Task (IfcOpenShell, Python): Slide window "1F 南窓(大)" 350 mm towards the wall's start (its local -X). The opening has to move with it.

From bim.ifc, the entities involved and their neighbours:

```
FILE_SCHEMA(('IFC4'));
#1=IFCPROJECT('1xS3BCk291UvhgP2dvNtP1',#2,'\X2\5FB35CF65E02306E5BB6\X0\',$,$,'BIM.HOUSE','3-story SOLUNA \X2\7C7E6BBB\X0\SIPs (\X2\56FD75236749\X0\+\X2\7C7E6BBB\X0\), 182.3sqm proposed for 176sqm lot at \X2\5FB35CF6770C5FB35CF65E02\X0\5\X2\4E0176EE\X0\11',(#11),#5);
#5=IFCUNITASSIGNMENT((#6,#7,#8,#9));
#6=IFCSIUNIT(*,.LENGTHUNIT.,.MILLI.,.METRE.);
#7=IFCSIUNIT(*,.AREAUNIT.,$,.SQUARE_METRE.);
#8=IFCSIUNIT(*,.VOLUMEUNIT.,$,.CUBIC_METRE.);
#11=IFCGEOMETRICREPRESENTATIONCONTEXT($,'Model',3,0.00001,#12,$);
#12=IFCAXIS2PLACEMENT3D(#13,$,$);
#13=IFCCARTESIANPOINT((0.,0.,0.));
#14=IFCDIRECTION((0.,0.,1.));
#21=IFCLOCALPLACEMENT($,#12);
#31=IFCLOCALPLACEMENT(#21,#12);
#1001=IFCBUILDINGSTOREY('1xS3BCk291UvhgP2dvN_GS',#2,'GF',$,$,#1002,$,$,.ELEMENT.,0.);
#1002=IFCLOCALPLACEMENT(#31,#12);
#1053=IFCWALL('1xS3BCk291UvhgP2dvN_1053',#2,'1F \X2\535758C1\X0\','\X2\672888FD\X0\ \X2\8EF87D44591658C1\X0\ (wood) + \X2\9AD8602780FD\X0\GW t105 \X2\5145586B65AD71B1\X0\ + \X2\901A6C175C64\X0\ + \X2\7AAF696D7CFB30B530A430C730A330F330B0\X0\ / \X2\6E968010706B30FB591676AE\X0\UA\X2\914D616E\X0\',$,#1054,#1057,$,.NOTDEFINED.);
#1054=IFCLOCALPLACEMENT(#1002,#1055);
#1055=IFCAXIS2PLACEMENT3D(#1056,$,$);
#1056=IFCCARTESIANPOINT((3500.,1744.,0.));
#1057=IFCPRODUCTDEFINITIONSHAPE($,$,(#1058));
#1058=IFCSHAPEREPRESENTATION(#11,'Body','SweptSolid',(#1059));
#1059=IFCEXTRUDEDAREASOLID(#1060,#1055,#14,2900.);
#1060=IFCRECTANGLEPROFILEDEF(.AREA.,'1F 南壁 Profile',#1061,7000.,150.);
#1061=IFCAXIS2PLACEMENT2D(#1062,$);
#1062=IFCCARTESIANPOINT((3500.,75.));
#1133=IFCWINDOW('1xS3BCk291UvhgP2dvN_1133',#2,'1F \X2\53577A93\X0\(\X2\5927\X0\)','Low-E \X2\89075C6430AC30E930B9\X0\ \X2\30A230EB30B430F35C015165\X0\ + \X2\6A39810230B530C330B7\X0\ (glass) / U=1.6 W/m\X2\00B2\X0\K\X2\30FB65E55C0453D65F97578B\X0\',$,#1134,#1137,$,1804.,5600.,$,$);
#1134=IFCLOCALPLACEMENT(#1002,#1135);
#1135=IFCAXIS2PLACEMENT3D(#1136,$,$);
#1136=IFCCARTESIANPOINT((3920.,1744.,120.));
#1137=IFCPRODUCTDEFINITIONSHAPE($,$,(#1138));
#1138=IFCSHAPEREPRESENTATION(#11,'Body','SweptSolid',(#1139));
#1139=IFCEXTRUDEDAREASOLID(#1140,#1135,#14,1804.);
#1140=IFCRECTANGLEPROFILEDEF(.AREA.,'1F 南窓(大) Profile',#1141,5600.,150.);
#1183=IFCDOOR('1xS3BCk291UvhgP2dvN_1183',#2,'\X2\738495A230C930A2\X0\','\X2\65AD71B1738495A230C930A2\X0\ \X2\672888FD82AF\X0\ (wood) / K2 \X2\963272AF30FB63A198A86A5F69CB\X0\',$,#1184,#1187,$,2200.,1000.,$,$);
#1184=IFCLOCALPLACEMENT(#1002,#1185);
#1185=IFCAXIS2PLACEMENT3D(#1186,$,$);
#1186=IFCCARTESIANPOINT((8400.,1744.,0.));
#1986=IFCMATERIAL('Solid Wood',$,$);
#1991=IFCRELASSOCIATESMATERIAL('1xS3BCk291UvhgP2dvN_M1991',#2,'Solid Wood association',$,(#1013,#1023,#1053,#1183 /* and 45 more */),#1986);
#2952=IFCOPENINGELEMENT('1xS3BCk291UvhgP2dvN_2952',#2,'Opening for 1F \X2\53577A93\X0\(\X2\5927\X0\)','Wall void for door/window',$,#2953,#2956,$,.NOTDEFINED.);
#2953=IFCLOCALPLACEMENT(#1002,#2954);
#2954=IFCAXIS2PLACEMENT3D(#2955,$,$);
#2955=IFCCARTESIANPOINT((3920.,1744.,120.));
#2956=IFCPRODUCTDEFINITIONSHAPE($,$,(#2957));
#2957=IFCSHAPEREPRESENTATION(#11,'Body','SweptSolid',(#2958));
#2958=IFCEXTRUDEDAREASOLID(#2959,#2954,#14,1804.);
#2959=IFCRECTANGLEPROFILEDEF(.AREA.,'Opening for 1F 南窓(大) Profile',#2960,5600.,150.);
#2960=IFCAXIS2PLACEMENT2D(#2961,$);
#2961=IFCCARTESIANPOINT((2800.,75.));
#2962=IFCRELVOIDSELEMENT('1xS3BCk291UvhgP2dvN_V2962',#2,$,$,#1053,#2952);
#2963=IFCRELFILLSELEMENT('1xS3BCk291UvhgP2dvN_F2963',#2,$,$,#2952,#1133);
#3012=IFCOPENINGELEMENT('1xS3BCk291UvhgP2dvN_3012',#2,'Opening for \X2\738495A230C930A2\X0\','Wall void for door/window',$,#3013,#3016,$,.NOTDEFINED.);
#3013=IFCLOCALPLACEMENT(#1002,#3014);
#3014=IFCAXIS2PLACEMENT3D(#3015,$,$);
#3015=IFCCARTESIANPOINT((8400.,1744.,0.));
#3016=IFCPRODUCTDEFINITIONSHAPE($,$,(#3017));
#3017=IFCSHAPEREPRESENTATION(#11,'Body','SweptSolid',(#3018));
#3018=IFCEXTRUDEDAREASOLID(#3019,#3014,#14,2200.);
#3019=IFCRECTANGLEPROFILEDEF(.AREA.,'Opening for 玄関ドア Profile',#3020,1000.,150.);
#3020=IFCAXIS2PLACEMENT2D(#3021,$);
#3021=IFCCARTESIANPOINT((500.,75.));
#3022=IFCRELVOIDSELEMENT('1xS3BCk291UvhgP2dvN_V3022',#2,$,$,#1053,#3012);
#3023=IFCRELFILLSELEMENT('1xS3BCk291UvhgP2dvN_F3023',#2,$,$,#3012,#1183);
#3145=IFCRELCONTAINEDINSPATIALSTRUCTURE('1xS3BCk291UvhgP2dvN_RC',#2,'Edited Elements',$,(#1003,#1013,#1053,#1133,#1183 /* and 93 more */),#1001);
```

```python
import ifcopenshell
import ifcopenshell.api.geometry
import ifcopenshell.util.placement

model = ifcopenshell.open("bim.ifc")

window = model.by_guid("1xS3BCk291UvhgP2dvN_1133")
opening = window.FillsVoids[0].RelatingOpeningElement
wall = opening.VoidsElements[0].RelatingBuildingElement

wall_matrix = ifcopenshell.util.placement.get_local_placement(wall.ObjectPlacement)
shift = wall_matrix[:3, 0] * -350.0
before = ifcopenshell.util.placement.get_local_placement(window.ObjectPlacement)[:3, 3].copy()

# The window is not placed relative to its opening, so move both.
for product in (opening, window):
    matrix = ifcopenshell.util.placement.get_local_placement(product.ObjectPlacement)
    matrix[:3, 3] += shift
    ifcopenshell.api.geometry.edit_object_placement(model, product=product, matrix=matrix, is_si=False)

after = ifcopenshell.util.placement.get_local_placement(window.ObjectPlacement)[:3, 3]
print("window moved by", (after - before).round(3) + 0.0)

model.write("bim_rev.ifc")
```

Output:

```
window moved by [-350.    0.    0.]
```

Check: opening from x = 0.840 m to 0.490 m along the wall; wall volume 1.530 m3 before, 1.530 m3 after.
